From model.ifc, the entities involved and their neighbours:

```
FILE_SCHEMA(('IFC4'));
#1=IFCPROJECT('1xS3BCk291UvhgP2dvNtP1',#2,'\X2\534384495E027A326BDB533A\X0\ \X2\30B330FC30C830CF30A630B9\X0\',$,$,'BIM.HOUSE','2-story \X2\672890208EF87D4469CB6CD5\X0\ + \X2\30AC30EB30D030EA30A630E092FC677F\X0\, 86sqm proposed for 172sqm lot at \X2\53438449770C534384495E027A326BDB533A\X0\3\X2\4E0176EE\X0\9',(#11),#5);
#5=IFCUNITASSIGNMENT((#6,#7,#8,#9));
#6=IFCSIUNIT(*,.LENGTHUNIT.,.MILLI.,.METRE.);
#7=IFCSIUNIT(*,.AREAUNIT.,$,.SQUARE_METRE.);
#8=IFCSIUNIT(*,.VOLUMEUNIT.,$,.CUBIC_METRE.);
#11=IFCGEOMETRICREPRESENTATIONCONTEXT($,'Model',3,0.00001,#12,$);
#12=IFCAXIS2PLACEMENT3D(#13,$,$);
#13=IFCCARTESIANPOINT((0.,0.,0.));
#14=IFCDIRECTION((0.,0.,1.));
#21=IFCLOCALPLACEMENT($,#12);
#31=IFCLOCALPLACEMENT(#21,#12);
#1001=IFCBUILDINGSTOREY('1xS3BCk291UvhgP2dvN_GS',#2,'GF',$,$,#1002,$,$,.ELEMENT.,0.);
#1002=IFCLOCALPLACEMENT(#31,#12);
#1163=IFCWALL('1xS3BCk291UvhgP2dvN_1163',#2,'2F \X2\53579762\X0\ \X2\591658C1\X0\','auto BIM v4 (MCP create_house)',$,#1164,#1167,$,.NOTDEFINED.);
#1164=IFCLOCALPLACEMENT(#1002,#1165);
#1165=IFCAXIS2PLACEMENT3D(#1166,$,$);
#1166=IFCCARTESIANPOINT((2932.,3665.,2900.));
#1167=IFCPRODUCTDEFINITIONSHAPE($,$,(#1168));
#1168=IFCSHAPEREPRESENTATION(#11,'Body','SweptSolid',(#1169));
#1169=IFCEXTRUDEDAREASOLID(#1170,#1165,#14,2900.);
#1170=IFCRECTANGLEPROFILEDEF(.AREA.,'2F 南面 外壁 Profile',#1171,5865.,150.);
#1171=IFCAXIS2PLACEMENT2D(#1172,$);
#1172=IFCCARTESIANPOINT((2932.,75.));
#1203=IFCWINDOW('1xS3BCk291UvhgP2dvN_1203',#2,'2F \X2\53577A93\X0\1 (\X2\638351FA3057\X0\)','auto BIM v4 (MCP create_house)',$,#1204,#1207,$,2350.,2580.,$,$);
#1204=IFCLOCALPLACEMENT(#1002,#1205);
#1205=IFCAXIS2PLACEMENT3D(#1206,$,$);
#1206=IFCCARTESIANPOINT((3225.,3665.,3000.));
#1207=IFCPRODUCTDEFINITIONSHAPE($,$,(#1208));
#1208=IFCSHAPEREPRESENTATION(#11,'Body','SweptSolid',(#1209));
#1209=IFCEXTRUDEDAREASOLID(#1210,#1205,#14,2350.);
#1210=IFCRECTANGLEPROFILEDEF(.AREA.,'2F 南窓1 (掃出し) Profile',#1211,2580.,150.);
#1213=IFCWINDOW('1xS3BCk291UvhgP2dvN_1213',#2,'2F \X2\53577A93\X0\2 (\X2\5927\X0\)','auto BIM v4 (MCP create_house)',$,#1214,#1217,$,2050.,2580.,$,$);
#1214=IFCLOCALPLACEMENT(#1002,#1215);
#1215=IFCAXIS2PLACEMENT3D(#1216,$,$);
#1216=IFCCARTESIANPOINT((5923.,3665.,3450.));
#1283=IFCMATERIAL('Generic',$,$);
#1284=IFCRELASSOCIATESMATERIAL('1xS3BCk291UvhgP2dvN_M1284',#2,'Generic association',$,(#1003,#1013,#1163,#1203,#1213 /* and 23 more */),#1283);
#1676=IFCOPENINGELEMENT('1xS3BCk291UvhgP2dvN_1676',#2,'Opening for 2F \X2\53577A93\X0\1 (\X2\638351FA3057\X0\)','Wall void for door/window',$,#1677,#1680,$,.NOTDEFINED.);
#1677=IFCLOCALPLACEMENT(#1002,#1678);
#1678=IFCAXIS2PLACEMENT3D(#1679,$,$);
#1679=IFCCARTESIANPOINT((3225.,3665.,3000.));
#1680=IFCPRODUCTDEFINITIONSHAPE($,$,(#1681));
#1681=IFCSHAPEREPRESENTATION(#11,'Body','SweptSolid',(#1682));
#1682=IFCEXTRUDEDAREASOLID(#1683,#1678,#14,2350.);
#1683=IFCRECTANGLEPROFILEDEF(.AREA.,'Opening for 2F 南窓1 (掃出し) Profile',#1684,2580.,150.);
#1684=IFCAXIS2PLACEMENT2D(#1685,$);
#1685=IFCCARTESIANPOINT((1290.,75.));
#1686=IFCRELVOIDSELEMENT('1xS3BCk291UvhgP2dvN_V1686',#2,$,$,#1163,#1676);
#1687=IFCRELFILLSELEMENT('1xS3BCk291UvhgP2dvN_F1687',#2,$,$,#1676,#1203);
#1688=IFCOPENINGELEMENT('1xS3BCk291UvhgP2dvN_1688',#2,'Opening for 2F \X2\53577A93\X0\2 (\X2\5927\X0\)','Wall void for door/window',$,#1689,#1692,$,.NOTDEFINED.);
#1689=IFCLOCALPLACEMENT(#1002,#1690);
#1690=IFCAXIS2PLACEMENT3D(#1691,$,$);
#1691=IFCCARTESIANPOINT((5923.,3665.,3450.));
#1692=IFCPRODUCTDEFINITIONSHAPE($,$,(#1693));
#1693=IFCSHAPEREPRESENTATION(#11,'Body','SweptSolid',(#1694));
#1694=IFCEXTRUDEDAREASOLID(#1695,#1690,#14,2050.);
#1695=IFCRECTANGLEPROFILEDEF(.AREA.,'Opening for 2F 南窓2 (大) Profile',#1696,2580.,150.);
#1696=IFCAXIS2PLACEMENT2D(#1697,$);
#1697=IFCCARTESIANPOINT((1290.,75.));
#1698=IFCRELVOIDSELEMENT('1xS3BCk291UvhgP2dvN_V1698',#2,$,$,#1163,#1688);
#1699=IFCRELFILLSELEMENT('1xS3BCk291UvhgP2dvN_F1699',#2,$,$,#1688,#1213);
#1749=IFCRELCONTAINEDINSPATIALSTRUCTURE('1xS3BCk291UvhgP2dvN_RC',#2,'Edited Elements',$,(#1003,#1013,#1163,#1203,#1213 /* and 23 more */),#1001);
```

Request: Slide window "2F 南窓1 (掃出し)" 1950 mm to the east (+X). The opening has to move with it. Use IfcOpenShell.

```python
import ifcopenshell
import ifcopenshell.api.geometry
import ifcopenshell.util.placement
import ifcopenshell.util.unit

model = ifcopenshell.open("model.ifc")
unit_scale = ifcopenshell.util.unit.calculate_unit_scale(model)

window = model.by_guid("1xS3BCk291UvhgP2dvN_1203")
opening = window.FillsVoids[0].RelatingOpeningElement
wall = opening.VoidsElements[0].RelatingBuildingElement

wall_matrix = ifcopenshell.util.placement.get_local_placement(wall.ObjectPlacement)
shift = wall_matrix[:3, 0] * 1.95 / unit_scale
before = ifcopenshell.util.placement.get_local_placement(window.ObjectPlacement)[:3, 3].copy()

# The window is not placed relative to its opening, so move both.
for product in (opening, window):
    matrix = ifcopenshell.util.placement.get_local_placement(product.ObjectPlacement)
    matrix[:3, 3] += shift
    ifcopenshell.api.geometry.edit_object_placement(model, product=product, matrix=matrix, is_si=False)

after = ifcopenshell.util.placement.get_local_placement(window.ObjectPlacement)[:3, 3]
print("window moved by", (after - before).round(3) + 0.0)

model.write("model_rev.ifc")
```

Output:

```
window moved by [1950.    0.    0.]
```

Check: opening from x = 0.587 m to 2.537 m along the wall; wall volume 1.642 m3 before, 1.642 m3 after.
